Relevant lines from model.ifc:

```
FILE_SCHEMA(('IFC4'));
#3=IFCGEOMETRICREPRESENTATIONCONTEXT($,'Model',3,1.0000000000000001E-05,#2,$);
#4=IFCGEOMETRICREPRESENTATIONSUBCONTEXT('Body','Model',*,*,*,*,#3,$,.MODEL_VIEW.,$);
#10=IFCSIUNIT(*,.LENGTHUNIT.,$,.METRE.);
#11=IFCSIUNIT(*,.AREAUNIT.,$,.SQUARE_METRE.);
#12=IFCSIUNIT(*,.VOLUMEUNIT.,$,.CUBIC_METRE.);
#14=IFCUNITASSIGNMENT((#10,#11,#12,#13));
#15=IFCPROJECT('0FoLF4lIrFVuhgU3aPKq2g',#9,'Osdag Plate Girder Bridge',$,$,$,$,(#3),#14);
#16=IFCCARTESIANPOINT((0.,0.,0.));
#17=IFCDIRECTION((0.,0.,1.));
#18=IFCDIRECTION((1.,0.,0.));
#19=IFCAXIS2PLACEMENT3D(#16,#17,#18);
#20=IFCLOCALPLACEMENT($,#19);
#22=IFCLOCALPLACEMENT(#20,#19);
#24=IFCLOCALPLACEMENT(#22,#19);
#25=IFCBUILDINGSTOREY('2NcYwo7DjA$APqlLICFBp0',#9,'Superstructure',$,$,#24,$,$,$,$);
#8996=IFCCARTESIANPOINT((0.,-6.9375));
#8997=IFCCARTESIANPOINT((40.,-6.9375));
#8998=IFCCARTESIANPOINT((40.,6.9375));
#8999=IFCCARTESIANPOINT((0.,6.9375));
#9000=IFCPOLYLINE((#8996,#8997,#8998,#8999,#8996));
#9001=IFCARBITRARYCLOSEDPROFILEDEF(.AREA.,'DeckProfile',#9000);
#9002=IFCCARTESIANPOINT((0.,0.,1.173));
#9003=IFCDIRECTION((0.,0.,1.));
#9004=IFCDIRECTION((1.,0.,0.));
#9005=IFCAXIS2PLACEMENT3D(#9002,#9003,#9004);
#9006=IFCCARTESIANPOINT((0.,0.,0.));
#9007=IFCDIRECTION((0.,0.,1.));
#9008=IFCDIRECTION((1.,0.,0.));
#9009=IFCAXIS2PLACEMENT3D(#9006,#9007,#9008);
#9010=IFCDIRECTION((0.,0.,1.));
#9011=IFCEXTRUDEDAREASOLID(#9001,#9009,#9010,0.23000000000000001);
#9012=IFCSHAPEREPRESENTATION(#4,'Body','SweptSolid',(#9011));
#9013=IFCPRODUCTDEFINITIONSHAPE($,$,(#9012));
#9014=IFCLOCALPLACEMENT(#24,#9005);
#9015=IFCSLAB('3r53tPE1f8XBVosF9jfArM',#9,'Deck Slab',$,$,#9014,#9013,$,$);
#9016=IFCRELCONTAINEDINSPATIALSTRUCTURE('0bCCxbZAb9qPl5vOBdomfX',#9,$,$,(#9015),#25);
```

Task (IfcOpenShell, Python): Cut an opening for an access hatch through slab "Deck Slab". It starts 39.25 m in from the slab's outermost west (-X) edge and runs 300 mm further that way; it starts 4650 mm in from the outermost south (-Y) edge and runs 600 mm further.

```python
import numpy as np
import ifcopenshell
import ifcopenshell.api.feature
import ifcopenshell.api.geometry
import ifcopenshell.api.root
import ifcopenshell.geom
import ifcopenshell.util.placement
import ifcopenshell.util.representation
import ifcopenshell.util.shape
import ifcopenshell.util.unit

model = ifcopenshell.open("model.ifc")
unit_scale = ifcopenshell.util.unit.calculate_unit_scale(model)
settings = ifcopenshell.geom.settings()


def volume(element):
    """Net volume in cubic metres, openings subtracted."""
    shape = ifcopenshell.geom.create_shape(settings, element)
    return ifcopenshell.util.shape.get_volume(shape.geometry)


slab = model.by_guid("3r53tPE1f8XBVosF9jfArM")
before = volume(slab)

# Extent in the slab's own axes, in metres. The edges named are its -X and -Y sides.
slab_shape = ifcopenshell.geom.create_shape(settings, slab)
vertices = ifcopenshell.util.shape.get_vertices(slab_shape.geometry)
x_min, y_min, bottom = vertices.min(axis=0)
top = vertices[:, 2].max()

opening = ifcopenshell.api.root.create_entity(model, ifc_class="IfcOpeningElement", name="Access hatch opening", predefined_type="OPENING")
context = ifcopenshell.util.representation.get_context(model, "Model", "Body", "MODEL_VIEW")
width, depth = 0.3, 0.6
outline = [(0.0, 0.0), (width, 0.0), (width, depth), (0.0, depth), (0.0, 0.0)]
# Overshoot both faces by 50 mm so the cut is clean.
shape = ifcopenshell.api.geometry.add_slab_representation(
    model, context=context, depth=top - bottom + 0.1, polyline=outline
)
ifcopenshell.api.geometry.assign_representation(model, product=opening, representation=shape)

matrix = ifcopenshell.util.placement.get_local_placement(slab.ObjectPlacement)
matrix[:, 3] = matrix @ np.append(np.array([x_min + 39.25, y_min + 4.65, bottom - 0.05]) / unit_scale, 1.0)
ifcopenshell.api.geometry.edit_object_placement(model, product=opening, matrix=matrix, is_si=False)
ifcopenshell.api.feature.add_feature(model, feature=opening, element=slab)

after = volume(slab)

print(f"slab volume {before:.3f} -> {after:.3f} m3")

model.write("model_v2.ifc")
```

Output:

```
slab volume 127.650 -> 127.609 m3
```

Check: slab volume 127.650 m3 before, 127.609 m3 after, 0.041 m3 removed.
